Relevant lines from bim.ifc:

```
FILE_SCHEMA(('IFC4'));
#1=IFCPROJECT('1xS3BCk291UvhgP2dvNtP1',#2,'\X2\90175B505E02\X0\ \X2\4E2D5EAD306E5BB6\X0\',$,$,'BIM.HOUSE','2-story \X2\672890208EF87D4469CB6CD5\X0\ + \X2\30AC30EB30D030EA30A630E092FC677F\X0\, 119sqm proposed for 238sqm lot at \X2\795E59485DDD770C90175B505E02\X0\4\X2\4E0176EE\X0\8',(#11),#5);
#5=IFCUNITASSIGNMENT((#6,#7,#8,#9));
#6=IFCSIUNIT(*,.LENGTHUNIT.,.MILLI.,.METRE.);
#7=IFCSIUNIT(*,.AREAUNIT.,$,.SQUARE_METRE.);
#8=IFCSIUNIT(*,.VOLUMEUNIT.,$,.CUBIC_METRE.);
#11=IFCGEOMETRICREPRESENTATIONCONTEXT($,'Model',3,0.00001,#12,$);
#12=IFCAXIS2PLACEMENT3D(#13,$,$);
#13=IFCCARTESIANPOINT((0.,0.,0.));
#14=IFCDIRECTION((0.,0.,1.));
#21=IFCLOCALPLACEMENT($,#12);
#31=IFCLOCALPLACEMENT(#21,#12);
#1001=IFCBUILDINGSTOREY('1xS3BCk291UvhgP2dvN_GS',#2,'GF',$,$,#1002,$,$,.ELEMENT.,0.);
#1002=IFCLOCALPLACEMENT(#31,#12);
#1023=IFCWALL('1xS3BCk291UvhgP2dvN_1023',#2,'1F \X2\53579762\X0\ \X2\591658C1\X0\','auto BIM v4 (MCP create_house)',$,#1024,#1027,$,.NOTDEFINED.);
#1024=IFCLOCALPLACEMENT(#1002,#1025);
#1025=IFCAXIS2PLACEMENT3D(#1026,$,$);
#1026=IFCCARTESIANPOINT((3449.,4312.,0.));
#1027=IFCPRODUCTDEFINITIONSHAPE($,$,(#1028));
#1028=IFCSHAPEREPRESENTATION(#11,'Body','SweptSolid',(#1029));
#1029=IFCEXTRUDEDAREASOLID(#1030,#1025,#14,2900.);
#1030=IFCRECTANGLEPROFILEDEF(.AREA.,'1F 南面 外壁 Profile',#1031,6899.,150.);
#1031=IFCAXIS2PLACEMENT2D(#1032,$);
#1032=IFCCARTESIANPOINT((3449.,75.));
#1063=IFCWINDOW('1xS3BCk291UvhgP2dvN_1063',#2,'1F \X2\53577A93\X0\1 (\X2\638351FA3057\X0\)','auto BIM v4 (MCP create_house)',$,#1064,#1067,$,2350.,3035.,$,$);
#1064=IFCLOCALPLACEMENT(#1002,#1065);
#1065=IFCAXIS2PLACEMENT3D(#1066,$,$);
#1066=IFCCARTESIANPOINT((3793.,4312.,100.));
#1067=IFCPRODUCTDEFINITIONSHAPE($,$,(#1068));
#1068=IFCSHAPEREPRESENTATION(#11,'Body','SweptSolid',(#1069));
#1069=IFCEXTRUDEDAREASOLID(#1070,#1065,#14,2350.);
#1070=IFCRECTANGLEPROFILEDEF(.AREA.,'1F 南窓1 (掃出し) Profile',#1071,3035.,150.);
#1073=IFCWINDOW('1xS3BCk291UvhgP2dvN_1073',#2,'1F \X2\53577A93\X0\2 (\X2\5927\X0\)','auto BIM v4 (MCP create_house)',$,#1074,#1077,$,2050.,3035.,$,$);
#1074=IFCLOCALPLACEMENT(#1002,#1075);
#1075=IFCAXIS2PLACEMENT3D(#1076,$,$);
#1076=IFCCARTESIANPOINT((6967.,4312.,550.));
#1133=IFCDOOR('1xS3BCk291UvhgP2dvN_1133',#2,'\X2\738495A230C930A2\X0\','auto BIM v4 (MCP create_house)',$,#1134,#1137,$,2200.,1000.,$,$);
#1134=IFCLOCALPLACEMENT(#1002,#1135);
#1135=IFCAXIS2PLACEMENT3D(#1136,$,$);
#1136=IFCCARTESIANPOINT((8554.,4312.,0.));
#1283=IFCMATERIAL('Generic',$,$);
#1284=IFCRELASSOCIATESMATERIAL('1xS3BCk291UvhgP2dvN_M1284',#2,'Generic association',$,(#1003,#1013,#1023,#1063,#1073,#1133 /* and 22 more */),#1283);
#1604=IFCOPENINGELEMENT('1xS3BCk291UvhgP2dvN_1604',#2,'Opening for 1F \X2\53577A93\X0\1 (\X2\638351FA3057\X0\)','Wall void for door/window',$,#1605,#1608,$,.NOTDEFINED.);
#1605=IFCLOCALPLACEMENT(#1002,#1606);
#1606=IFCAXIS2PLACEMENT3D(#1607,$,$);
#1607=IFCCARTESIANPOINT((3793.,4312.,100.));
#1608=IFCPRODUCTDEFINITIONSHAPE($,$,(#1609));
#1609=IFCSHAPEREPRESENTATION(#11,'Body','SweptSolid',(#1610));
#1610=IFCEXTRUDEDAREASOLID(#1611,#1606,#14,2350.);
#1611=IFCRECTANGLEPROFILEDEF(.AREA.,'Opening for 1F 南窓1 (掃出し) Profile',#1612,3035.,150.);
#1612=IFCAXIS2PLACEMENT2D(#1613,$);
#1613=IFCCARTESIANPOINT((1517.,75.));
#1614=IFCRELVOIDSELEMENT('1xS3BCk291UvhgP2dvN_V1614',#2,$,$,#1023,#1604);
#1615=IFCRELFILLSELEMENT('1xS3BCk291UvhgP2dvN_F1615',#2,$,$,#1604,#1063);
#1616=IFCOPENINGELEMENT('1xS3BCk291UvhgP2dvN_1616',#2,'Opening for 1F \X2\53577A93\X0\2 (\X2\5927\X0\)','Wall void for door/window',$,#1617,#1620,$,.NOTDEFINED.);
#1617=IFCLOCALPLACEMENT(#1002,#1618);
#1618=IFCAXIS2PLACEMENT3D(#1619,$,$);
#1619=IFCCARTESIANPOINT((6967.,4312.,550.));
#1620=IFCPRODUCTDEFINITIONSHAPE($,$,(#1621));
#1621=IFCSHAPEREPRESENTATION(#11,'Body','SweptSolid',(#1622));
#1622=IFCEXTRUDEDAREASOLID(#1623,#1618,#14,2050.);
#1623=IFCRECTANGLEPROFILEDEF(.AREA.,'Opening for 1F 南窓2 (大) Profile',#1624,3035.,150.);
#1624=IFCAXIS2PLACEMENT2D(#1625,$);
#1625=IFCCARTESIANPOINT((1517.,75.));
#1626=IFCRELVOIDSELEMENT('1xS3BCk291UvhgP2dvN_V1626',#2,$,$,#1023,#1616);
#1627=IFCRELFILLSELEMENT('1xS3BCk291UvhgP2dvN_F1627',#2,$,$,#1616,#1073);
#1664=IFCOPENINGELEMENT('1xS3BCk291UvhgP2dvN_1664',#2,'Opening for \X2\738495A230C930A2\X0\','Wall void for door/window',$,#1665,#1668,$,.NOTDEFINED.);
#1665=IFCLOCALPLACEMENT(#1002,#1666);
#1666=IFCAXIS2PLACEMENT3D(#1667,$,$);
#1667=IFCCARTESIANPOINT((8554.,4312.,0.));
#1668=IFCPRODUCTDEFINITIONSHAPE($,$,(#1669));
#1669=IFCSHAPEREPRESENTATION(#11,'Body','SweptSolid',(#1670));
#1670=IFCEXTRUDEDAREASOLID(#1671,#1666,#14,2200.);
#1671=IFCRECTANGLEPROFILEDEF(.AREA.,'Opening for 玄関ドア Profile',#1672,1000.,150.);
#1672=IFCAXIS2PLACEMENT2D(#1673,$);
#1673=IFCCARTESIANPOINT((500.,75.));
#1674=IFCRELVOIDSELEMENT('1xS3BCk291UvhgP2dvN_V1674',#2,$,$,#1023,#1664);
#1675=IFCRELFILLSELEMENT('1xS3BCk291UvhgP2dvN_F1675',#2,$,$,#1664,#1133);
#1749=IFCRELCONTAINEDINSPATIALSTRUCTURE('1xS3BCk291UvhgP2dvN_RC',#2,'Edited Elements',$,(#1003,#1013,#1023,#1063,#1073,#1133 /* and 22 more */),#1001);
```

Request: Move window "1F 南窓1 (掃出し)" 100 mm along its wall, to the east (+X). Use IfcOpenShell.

```python
import ifcopenshell
import ifcopenshell.api.geometry
import ifcopenshell.util.placement
import ifcopenshell.util.unit

model = ifcopenshell.open("bim.ifc")
unit_scale = ifcopenshell.util.unit.calculate_unit_scale(model)

window = model.by_id(1063)
opening = window.FillsVoids[0].RelatingOpeningElement
wall = opening.VoidsElements[0].RelatingBuildingElement

wall_matrix = ifcopenshell.util.placement.get_local_placement(wall.ObjectPlacement)
shift = wall_matrix[:3, 0] * 0.1 / unit_scale
before = ifcopenshell.util.placement.get_local_placement(window.ObjectPlacement)[:3, 3].copy()

# The window is not placed relative to its opening, so move both.
for product in (opening, window):
    matrix = ifcopenshell.util.placement.get_local_placement(product.ObjectPlacement)
    matrix[:3, 3] += shift
    ifcopenshell.api.geometry.edit_object_placement(model, product=product, matrix=matrix, is_si=False)

after = ifcopenshell.util.placement.get_local_placement(window.ObjectPlacement)[:3, 3]
print("window moved by", (after - before).round(3) + 0.0)

model.write("bim_v2.ifc")
```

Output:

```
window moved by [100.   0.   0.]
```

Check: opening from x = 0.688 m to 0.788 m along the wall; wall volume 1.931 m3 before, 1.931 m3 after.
